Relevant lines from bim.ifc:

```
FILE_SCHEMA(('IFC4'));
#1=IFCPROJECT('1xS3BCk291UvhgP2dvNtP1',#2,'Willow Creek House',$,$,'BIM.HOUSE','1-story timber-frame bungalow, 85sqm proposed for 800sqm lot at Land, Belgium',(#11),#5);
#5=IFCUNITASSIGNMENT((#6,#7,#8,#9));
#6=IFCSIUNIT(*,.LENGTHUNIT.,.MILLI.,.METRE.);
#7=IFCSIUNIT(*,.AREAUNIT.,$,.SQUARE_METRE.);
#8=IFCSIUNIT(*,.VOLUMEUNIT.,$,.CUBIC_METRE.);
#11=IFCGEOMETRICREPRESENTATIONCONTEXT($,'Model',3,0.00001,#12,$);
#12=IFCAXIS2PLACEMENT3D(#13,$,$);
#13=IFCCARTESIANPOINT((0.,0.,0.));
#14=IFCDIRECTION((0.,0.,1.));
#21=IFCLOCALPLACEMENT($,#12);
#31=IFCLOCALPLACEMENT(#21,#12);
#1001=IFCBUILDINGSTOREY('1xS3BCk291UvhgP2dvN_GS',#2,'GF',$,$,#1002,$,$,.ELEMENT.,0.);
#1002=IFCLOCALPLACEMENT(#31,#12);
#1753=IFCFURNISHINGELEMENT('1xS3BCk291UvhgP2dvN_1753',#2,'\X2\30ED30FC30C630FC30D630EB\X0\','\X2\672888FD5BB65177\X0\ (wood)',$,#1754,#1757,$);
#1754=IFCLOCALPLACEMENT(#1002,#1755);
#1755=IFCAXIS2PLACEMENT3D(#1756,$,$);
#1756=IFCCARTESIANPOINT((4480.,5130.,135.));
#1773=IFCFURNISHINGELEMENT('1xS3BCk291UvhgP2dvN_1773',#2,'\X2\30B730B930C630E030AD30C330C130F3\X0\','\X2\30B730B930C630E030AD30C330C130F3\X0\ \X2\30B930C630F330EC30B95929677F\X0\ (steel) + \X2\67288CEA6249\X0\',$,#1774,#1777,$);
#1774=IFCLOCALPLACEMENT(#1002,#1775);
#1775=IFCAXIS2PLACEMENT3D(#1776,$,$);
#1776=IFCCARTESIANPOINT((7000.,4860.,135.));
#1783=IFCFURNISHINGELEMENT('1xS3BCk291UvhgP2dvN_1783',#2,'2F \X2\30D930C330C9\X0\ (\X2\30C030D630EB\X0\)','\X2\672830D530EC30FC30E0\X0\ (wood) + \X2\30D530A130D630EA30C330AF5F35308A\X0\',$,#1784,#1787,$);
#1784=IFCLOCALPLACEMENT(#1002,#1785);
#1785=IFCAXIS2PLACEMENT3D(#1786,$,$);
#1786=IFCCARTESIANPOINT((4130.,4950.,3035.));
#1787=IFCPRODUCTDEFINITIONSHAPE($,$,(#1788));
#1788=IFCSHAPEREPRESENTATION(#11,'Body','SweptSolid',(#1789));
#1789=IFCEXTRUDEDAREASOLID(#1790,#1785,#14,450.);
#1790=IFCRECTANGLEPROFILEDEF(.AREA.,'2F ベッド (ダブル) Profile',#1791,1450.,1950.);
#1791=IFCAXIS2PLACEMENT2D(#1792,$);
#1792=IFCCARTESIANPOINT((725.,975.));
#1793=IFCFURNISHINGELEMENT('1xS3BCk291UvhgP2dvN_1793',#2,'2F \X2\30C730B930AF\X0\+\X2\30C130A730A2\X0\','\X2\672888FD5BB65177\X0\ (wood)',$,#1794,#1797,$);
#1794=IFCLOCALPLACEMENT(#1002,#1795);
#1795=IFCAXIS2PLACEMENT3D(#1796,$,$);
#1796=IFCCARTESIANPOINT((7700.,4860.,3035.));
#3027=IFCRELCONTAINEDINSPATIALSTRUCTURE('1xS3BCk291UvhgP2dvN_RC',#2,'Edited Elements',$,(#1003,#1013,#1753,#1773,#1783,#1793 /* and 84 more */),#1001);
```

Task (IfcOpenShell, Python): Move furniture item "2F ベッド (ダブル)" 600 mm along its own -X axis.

```python
import ifcopenshell
import ifcopenshell.api.geometry
import ifcopenshell.util.placement
import ifcopenshell.util.unit

model = ifcopenshell.open("bim.ifc")
unit_scale = ifcopenshell.util.unit.calculate_unit_scale(model)

item = model.by_guid("1xS3BCk291UvhgP2dvN_1783")
matrix = ifcopenshell.util.placement.get_local_placement(item.ObjectPlacement)
matrix[:3, 3] -= matrix[:3, 0] * 0.6 / unit_scale
ifcopenshell.api.geometry.edit_object_placement(model, product=item, matrix=matrix, is_si=False)

print(ifcopenshell.util.placement.get_local_placement(item.ObjectPlacement).round(3) + 0.0)

model.write("bim_edited.ifc")
```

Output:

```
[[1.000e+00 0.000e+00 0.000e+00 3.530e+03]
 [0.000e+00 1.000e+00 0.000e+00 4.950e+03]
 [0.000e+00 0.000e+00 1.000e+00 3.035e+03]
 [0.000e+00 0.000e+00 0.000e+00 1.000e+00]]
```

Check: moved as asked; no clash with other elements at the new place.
